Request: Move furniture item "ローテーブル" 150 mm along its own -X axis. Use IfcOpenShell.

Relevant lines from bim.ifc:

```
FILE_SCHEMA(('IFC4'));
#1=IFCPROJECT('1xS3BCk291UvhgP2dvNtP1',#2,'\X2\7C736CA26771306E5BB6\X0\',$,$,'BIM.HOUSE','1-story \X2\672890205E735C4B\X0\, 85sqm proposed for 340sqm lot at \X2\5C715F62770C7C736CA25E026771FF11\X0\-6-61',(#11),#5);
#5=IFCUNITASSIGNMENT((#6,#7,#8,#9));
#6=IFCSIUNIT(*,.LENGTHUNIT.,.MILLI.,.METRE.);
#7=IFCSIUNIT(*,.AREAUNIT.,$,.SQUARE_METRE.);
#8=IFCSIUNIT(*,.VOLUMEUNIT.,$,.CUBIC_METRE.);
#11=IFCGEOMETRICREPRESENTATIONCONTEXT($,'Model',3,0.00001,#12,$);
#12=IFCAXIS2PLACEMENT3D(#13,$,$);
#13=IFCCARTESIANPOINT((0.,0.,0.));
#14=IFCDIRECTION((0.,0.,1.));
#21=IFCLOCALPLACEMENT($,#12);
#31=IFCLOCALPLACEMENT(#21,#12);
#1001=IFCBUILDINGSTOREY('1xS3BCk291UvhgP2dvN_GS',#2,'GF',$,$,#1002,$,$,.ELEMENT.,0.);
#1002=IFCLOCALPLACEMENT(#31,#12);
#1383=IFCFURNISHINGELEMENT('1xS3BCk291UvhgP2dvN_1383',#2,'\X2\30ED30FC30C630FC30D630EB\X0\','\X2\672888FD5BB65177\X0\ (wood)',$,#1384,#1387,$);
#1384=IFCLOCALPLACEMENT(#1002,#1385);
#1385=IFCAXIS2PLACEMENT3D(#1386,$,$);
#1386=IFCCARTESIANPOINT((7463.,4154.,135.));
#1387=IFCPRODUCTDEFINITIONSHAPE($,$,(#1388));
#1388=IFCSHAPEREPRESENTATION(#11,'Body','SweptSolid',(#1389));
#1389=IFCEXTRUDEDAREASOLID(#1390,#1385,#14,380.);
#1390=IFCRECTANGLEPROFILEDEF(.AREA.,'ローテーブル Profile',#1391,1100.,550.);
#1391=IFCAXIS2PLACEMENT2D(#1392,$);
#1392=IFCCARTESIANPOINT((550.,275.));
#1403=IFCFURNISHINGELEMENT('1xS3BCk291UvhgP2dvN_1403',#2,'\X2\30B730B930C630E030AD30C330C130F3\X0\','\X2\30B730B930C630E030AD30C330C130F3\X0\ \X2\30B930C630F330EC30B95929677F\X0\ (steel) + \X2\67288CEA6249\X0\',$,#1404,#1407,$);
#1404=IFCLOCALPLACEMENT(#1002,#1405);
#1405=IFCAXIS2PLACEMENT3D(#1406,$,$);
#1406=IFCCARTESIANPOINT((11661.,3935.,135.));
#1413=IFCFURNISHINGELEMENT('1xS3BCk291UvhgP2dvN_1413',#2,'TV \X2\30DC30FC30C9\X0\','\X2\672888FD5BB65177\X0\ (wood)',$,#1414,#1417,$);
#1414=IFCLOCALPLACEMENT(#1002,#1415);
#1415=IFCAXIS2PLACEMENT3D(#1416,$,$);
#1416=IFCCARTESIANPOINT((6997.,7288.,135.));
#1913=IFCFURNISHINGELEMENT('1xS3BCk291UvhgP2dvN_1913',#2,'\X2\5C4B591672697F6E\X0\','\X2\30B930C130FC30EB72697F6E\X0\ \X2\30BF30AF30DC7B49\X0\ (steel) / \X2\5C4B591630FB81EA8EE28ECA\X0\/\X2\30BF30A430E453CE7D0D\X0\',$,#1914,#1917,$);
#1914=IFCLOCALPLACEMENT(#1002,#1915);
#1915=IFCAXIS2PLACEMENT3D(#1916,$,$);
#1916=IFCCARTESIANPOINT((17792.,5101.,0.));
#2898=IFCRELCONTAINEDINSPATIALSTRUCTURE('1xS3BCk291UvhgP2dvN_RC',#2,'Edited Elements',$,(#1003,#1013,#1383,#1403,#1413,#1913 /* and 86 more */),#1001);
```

```python
import ifcopenshell
import ifcopenshell.api.geometry
import ifcopenshell.util.placement
import ifcopenshell.util.unit

model = ifcopenshell.open("bim.ifc")
unit_scale = ifcopenshell.util.unit.calculate_unit_scale(model)

item = model.by_guid("1xS3BCk291UvhgP2dvN_1383")
matrix = ifcopenshell.util.placement.get_local_placement(item.ObjectPlacement)
matrix[:3, 3] -= matrix[:3, 0] * 0.15 / unit_scale
ifcopenshell.api.geometry.edit_object_placement(model, product=item, matrix=matrix, is_si=False)

print(ifcopenshell.util.placement.get_local_placement(item.ObjectPlacement).round(3) + 0.0)

model.write("bim_rev.ifc")
```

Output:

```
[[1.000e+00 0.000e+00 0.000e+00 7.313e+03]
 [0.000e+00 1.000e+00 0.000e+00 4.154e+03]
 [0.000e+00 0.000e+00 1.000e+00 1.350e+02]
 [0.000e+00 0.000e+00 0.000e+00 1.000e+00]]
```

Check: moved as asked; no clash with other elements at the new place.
